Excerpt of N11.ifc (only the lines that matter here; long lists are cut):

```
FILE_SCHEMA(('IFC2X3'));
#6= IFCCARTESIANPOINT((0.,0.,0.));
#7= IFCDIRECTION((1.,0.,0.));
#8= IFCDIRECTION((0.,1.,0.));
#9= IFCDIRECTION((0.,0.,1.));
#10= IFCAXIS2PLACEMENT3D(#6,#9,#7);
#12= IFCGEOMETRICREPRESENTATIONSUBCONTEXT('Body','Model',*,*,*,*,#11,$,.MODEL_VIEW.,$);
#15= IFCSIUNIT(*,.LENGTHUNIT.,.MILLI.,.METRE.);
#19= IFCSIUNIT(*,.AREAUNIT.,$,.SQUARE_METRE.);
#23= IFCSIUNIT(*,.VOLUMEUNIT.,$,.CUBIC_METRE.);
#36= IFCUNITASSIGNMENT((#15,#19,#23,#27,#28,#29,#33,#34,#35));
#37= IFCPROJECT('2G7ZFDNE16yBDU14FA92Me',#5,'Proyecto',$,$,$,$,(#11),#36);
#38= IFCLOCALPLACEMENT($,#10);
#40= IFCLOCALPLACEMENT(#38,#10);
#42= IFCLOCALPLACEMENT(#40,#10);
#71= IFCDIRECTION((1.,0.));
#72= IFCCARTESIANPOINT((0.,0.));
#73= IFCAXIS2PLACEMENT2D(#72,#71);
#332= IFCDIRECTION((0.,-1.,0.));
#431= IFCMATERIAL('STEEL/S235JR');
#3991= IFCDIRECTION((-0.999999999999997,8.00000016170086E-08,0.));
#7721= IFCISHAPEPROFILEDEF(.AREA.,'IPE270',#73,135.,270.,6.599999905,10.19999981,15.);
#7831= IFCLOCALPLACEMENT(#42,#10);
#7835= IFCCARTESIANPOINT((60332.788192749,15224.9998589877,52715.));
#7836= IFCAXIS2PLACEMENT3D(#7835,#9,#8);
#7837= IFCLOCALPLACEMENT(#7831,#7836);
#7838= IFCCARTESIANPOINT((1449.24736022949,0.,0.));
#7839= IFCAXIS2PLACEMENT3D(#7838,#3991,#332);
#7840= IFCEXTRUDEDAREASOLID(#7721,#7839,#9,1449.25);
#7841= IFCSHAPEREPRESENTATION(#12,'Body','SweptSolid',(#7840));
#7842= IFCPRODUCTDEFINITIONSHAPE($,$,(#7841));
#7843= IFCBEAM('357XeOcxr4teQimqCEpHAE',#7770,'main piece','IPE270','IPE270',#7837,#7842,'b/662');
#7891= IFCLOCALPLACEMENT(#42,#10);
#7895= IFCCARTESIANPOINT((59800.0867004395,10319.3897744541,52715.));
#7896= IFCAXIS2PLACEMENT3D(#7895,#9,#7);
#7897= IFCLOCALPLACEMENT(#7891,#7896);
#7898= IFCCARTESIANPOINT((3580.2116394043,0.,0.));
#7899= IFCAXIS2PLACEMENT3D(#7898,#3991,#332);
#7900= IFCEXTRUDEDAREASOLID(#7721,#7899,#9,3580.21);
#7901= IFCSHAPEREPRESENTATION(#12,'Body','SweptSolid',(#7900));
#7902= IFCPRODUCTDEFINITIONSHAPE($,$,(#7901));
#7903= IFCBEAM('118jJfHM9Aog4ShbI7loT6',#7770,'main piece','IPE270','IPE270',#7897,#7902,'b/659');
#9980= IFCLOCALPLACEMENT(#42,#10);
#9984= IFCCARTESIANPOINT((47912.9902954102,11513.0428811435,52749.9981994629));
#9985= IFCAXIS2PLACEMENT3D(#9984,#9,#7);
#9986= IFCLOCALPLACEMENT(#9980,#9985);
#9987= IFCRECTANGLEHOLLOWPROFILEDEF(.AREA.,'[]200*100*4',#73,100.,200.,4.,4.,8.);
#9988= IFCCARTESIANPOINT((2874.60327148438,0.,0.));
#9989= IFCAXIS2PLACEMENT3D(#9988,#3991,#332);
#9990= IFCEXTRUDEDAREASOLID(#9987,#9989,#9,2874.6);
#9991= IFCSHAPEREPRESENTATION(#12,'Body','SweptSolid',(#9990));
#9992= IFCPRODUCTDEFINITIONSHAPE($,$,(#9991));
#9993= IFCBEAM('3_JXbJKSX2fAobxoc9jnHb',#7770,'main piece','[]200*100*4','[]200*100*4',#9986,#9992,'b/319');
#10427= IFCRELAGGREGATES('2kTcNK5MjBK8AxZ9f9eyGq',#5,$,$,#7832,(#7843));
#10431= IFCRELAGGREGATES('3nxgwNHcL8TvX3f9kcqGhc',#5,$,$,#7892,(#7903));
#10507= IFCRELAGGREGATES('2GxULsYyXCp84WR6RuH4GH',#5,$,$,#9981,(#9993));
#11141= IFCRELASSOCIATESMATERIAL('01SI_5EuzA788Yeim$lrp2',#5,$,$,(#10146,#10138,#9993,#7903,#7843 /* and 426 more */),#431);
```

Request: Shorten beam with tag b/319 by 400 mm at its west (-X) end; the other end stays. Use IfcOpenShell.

```python
import ifcopenshell
import ifcopenshell.util.representation

model = ifcopenshell.open("N11.ifc")

member = model.by_id(9993)
change = -400.0

# The extrusion runs towards the end named, so only its depth changes.
body = ifcopenshell.util.representation.get_representation(member, "Model", "Body")
solid = body.Items[0]
old_length = solid.Depth
solid.Depth += change

print(f"length {old_length:g} -> {solid.Depth:g}")

model.write("N11_updated.ifc")
```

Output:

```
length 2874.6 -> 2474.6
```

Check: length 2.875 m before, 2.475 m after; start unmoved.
